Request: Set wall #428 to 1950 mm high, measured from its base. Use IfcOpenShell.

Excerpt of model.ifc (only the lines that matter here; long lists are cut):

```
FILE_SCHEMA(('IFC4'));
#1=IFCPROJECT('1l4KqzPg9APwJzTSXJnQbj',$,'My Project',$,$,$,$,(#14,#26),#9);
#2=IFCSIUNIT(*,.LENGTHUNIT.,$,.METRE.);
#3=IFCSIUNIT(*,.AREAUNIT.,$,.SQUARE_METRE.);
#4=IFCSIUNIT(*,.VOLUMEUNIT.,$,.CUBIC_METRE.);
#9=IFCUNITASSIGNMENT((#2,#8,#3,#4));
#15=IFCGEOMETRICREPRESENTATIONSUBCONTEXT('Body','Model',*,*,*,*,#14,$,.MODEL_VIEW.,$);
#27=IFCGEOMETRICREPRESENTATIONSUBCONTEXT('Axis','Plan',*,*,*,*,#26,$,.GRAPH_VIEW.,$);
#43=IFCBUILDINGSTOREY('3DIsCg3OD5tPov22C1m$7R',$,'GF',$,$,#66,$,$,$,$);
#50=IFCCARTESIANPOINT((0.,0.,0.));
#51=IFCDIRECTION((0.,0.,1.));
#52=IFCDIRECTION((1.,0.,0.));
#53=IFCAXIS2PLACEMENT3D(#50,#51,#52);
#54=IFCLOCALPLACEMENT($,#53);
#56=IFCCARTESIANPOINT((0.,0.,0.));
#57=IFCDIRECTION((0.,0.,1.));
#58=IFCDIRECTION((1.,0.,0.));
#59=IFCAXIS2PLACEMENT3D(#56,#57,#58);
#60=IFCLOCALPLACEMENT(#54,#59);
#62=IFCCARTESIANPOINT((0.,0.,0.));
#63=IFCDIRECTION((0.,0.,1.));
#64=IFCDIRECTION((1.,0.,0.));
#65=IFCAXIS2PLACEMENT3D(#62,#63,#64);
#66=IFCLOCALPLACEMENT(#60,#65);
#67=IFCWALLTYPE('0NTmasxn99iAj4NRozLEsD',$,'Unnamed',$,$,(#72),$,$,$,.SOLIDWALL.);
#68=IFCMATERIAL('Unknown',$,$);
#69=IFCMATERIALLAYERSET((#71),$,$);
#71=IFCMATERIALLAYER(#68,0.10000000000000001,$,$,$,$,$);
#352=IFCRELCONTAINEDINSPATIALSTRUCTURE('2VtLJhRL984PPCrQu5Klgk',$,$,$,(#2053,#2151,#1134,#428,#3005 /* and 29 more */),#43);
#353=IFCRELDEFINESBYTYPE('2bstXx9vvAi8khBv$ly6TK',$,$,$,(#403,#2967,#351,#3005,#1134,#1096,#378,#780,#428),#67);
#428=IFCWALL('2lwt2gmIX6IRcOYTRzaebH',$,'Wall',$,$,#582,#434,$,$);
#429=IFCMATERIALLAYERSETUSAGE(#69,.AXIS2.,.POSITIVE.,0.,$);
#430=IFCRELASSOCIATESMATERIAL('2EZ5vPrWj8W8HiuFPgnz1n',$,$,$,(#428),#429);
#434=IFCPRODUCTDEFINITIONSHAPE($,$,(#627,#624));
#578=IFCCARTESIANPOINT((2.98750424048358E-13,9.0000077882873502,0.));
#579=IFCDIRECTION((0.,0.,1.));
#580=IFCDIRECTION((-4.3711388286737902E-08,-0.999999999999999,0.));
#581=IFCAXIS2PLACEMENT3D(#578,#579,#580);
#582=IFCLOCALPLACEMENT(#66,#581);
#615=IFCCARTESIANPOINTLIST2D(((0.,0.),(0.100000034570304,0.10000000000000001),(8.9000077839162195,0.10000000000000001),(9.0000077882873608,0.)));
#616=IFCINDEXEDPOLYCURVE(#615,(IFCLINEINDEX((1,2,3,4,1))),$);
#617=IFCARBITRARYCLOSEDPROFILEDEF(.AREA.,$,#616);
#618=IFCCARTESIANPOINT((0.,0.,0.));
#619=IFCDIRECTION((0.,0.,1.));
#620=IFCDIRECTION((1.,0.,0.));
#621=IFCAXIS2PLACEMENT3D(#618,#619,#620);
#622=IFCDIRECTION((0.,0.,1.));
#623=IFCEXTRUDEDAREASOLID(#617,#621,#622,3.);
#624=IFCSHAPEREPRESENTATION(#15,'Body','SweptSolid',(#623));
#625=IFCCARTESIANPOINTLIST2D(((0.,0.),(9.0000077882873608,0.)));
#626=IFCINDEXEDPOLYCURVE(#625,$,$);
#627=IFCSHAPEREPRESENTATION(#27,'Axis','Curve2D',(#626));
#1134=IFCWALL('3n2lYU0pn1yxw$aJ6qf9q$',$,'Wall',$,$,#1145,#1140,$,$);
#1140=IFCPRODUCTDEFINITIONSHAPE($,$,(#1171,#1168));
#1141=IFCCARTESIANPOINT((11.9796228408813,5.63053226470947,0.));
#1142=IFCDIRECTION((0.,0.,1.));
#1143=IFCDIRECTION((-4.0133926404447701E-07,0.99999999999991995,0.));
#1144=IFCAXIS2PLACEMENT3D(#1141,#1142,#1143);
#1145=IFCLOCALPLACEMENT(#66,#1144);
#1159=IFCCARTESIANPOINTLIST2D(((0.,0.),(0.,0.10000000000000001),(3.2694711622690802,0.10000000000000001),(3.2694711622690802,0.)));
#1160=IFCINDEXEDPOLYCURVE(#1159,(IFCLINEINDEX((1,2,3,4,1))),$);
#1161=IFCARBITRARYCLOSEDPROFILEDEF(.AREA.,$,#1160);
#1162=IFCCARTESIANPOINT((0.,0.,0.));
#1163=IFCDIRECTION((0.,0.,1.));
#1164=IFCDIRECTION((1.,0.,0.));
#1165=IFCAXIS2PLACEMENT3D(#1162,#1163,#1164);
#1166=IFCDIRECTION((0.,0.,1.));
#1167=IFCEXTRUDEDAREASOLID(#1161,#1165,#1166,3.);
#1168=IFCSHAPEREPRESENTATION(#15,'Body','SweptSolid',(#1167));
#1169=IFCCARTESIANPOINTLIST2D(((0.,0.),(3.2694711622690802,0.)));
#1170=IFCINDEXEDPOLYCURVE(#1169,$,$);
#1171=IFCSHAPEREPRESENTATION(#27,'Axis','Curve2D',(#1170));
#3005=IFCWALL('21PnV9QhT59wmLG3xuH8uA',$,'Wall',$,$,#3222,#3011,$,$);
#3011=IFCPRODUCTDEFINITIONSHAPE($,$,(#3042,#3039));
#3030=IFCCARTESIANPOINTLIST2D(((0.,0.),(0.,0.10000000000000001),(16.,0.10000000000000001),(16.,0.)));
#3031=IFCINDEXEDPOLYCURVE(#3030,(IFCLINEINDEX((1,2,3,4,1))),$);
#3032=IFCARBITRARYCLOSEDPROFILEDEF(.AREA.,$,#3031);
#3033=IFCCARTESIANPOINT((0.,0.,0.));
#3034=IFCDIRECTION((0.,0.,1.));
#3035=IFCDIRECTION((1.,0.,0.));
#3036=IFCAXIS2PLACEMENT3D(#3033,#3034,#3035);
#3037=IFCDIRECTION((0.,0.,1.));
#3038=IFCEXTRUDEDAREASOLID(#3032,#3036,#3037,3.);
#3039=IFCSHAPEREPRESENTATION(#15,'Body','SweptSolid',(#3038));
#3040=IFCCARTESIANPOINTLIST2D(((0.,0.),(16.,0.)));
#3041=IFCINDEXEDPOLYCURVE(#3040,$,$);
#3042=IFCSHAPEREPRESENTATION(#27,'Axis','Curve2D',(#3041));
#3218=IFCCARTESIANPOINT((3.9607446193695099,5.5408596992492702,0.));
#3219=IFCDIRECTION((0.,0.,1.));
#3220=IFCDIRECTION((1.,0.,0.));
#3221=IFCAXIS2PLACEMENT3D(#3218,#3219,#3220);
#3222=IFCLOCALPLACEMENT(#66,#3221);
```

```python
import ifcopenshell
import ifcopenshell.geom
import ifcopenshell.util.representation
import ifcopenshell.util.shape
import ifcopenshell.util.unit

model = ifcopenshell.open("model.ifc")
unit_scale = ifcopenshell.util.unit.calculate_unit_scale(model)
settings = ifcopenshell.geom.settings()


def volume(element):
    """Net volume in cubic metres, openings subtracted."""
    shape = ifcopenshell.geom.create_shape(settings, element)
    return ifcopenshell.util.shape.get_volume(shape.geometry)


wall = model.by_id(428)
before = volume(wall)

body = ifcopenshell.util.representation.get_representation(wall, "Model", "Body")
solid = body.Items[0]
old_height = solid.Depth
solid.Depth = 1.95 / unit_scale
after = volume(wall)

print(f"height {old_height:g} -> {solid.Depth:g}, volume {before:.3f} -> {after:.3f} m3")

model.write("model_edited.ifc")
```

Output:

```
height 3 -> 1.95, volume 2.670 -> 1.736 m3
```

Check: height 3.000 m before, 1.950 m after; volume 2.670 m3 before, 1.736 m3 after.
